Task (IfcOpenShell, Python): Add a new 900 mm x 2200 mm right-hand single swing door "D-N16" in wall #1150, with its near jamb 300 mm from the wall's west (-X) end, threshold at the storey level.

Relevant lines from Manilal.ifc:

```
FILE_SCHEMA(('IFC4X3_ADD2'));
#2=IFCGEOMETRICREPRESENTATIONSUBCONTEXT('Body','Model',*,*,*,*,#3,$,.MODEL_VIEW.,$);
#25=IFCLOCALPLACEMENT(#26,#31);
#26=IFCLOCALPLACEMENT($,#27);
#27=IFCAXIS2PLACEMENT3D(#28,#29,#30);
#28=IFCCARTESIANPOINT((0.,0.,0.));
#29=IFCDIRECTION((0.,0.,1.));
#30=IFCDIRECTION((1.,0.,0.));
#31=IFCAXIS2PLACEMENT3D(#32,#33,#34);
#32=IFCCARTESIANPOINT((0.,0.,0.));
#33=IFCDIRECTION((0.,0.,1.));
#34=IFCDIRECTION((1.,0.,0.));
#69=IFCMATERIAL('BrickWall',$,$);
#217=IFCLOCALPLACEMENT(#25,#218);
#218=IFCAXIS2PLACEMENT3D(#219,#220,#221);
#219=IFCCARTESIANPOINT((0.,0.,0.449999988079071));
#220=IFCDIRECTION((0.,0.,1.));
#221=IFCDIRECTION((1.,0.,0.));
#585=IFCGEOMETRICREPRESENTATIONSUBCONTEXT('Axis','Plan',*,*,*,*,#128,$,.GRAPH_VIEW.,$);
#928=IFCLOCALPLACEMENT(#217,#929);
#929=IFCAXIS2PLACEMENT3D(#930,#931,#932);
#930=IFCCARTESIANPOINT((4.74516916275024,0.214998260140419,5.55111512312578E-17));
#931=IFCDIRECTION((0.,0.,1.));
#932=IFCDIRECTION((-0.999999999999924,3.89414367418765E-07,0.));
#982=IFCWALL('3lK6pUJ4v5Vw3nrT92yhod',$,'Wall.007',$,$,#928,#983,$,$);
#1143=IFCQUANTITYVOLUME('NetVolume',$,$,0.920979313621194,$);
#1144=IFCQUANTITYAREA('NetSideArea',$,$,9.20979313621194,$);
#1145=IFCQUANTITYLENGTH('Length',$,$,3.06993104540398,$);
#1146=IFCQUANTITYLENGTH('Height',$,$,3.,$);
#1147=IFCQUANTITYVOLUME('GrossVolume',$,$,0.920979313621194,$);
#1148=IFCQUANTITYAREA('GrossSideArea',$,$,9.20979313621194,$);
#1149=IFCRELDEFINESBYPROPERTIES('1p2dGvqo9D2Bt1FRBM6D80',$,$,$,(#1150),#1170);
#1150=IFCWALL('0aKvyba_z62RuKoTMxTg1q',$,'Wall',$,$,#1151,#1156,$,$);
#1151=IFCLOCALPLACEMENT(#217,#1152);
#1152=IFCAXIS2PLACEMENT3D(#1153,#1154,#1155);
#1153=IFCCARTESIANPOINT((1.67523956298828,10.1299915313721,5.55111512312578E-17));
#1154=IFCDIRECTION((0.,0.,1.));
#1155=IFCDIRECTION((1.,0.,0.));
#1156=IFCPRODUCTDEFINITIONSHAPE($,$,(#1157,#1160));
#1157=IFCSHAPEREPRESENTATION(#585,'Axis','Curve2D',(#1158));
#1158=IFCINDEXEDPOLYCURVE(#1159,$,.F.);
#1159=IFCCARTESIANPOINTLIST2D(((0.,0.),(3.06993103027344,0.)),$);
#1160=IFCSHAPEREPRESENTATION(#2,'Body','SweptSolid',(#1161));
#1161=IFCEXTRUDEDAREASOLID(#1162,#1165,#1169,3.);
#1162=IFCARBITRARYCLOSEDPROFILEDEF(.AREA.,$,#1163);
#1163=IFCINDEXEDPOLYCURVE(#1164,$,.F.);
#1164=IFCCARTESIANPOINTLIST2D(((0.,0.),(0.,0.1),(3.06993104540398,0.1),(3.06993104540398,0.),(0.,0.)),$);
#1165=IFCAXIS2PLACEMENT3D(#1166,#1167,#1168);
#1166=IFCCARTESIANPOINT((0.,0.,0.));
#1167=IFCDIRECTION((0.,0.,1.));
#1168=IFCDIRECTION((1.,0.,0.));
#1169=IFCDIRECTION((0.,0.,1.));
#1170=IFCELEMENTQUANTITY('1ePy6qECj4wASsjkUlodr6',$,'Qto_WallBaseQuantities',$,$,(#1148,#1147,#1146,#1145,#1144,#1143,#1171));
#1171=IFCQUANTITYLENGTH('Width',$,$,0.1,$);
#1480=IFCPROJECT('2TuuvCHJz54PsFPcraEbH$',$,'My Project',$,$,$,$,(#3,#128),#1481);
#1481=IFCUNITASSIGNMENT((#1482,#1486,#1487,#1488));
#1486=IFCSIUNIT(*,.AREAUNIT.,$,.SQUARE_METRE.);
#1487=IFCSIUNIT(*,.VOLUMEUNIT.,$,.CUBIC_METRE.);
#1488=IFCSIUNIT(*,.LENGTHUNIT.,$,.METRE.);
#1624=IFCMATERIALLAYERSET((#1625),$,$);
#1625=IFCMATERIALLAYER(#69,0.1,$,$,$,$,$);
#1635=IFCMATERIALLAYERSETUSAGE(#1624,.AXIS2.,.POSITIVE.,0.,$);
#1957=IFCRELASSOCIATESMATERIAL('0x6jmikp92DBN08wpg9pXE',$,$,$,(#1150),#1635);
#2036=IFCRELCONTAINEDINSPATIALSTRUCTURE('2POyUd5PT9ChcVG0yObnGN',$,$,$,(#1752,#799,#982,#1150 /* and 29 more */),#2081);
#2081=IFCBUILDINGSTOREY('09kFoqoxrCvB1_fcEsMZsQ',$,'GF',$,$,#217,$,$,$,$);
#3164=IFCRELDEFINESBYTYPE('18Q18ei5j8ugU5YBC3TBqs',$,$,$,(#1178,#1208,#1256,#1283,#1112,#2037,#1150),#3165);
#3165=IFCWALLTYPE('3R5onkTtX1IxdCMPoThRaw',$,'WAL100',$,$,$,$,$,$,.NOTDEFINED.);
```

```python
import numpy as np
import ifcopenshell
import ifcopenshell.api.feature
import ifcopenshell.api.geometry
import ifcopenshell.api.pset
import ifcopenshell.api.root
import ifcopenshell.api.spatial
import ifcopenshell.geom
import ifcopenshell.util.element
import ifcopenshell.util.placement
import ifcopenshell.util.representation
import ifcopenshell.util.shape
import ifcopenshell.util.unit

model = ifcopenshell.open("Manilal.ifc")
unit_scale = ifcopenshell.util.unit.calculate_unit_scale(model)
area_scale = ifcopenshell.util.unit.calculate_unit_scale(model, "AREAUNIT")
volume_scale = ifcopenshell.util.unit.calculate_unit_scale(model, "VOLUMEUNIT")
settings = ifcopenshell.geom.settings()


def volume(element):
    """Net volume in cubic metres, openings subtracted."""
    shape = ifcopenshell.geom.create_shape(settings, element)
    return ifcopenshell.util.shape.get_volume(shape.geometry)


wall = model.by_guid("0aKvyba_z62RuKoTMxTg1q")
storey = ifcopenshell.util.element.get_container(wall, ifc_class="IfcBuildingStorey")
context = ifcopenshell.util.representation.get_context(model, "Model", "Body", "MODEL_VIEW")
before = volume(wall)

width, height, from_end, sill = 0.9, 2.2, 0.3, 0.0  # metres

# The wall runs along its own X axis, and the end named is its -X end.
wall_shape = ifcopenshell.geom.create_shape(settings, wall)
x, y, z = ifcopenshell.util.shape.get_vertices(wall_shape.geometry).T
start = x.min() + from_end
face, thickness = float(y.min()), float(y.max() - y.min())
wall_matrix = ifcopenshell.util.placement.get_local_placement(wall.ObjectPlacement)
level = ifcopenshell.util.placement.get_local_placement(storey.ObjectPlacement)[2, 3]


def in_wall(x, y):
    """Placement at x, y metres in the wall's axes, at sill height."""
    matrix = wall_matrix.copy()
    matrix[:, 3] = wall_matrix @ np.array([x / unit_scale, y / unit_scale, 0.0, 1.0])
    matrix[2, 3] = level + sill / unit_scale
    return matrix


# Opening: a box that overshoots both wall faces by 50 mm.
opening = ifcopenshell.api.root.create_entity(model, ifc_class="IfcOpeningElement", predefined_type="OPENING")
box = ifcopenshell.api.geometry.add_wall_representation(
    model, context=context, length=width, height=height, thickness=thickness + 0.1
)
ifcopenshell.api.geometry.assign_representation(model, product=opening, representation=box)
ifcopenshell.api.geometry.edit_object_placement(model, product=opening, matrix=in_wall(start, face - 0.05), is_si=False)
ifcopenshell.api.feature.add_feature(model, feature=opening, element=wall)

door = ifcopenshell.api.root.create_entity(model, ifc_class="IfcDoor", name="D-N16", predefined_type="DOOR")
door.OverallWidth, door.OverallHeight = width / unit_scale, height / unit_scale
door.OperationType = "SINGLE_SWING_RIGHT"
body = ifcopenshell.api.geometry.add_door_representation(
    model,
    context=context,
    overall_width=door.OverallWidth,
    overall_height=door.OverallHeight,
    operation_type="SINGLE_SWING_RIGHT",
    lining_properties={"LiningDepth": thickness / unit_scale, "ThresholdDepth": thickness / unit_scale},
)
ifcopenshell.api.geometry.assign_representation(model, product=door, representation=body)
ifcopenshell.api.spatial.assign_container(model, products=[door], relating_structure=storey)
ifcopenshell.api.feature.add_filling(model, opening=opening, element=door)

# The lining spans the wall, so the door starts at the wall face.
ifcopenshell.api.geometry.edit_object_placement(model, product=door, matrix=in_wall(start, face), is_si=False)

after = volume(wall)

# Update the wall's stored quantities.
qto = model.by_id(ifcopenshell.util.element.get_pset(wall, "Qto_WallBaseQuantities", should_inherit=False)["id"])
ifcopenshell.api.pset.edit_qto(model, qto=qto, properties={
    "NetSideArea": after / thickness / area_scale,
    "NetVolume": after / volume_scale,
})

print(f"wall volume {before:.3f} -> {after:.3f} m3")

model.write("Manilal-out.ifc")
```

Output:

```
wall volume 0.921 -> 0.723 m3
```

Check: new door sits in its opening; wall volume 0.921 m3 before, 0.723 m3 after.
